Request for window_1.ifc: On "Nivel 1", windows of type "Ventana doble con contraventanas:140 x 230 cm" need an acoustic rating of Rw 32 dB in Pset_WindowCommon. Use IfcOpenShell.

First a look at what the model holds.

```python
import ifcopenshell
import ifcopenshell.util.element

model = ifcopenshell.open("window_1.ifc")
print(model.schema)
storey = next(s for s in model.by_type("IfcBuildingStorey") if s.Name == "Nivel 1")
windows = [e for e in ifcopenshell.util.element.get_decomposition(storey) if e.is_a("IfcWindow")]
seen = {}
for e in windows:
    element_type = ifcopenshell.util.element.get_type(e)
    key = (element_type.Name if element_type != e and element_type else None, ifcopenshell.util.element.get_pset(e, "Pset_WindowCommon", "AcousticRating"))
    seen[key] = seen.get(key, 0) + 1
for (name, value), count in sorted(seen.items(), key=str):
    print(count, "x", name, "|", value)
```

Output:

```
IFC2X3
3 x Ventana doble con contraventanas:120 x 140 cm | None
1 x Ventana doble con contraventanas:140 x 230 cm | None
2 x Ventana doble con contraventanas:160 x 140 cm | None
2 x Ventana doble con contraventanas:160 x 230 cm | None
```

```python
import ifcopenshell
import ifcopenshell.api.pset
import ifcopenshell.util.element

model = ifcopenshell.open("window_1.ifc")

storey = next(s for s in model.by_type("IfcBuildingStorey") if s.Name == "Nivel 1")
windows = [e for e in ifcopenshell.util.element.get_decomposition(storey) if e.is_a("IfcWindow")]

count = 0
for e in windows:
    element_type = ifcopenshell.util.element.get_type(e)
    if element_type in (None, e) or element_type.Name != "Ventana doble con contraventanas:140 x 230 cm":
        continue
    # add_pset returns the element's existing set when there is one.
    pset = ifcopenshell.api.pset.add_pset(model, product=e, name="Pset_WindowCommon")
    ifcopenshell.api.pset.edit_pset(model, pset=pset, properties={"AcousticRating": "Rw 32 dB"})
    count += 1

print(count, "windows updated")

model.write("window_1_v2.ifc")
```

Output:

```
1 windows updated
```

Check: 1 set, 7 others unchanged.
